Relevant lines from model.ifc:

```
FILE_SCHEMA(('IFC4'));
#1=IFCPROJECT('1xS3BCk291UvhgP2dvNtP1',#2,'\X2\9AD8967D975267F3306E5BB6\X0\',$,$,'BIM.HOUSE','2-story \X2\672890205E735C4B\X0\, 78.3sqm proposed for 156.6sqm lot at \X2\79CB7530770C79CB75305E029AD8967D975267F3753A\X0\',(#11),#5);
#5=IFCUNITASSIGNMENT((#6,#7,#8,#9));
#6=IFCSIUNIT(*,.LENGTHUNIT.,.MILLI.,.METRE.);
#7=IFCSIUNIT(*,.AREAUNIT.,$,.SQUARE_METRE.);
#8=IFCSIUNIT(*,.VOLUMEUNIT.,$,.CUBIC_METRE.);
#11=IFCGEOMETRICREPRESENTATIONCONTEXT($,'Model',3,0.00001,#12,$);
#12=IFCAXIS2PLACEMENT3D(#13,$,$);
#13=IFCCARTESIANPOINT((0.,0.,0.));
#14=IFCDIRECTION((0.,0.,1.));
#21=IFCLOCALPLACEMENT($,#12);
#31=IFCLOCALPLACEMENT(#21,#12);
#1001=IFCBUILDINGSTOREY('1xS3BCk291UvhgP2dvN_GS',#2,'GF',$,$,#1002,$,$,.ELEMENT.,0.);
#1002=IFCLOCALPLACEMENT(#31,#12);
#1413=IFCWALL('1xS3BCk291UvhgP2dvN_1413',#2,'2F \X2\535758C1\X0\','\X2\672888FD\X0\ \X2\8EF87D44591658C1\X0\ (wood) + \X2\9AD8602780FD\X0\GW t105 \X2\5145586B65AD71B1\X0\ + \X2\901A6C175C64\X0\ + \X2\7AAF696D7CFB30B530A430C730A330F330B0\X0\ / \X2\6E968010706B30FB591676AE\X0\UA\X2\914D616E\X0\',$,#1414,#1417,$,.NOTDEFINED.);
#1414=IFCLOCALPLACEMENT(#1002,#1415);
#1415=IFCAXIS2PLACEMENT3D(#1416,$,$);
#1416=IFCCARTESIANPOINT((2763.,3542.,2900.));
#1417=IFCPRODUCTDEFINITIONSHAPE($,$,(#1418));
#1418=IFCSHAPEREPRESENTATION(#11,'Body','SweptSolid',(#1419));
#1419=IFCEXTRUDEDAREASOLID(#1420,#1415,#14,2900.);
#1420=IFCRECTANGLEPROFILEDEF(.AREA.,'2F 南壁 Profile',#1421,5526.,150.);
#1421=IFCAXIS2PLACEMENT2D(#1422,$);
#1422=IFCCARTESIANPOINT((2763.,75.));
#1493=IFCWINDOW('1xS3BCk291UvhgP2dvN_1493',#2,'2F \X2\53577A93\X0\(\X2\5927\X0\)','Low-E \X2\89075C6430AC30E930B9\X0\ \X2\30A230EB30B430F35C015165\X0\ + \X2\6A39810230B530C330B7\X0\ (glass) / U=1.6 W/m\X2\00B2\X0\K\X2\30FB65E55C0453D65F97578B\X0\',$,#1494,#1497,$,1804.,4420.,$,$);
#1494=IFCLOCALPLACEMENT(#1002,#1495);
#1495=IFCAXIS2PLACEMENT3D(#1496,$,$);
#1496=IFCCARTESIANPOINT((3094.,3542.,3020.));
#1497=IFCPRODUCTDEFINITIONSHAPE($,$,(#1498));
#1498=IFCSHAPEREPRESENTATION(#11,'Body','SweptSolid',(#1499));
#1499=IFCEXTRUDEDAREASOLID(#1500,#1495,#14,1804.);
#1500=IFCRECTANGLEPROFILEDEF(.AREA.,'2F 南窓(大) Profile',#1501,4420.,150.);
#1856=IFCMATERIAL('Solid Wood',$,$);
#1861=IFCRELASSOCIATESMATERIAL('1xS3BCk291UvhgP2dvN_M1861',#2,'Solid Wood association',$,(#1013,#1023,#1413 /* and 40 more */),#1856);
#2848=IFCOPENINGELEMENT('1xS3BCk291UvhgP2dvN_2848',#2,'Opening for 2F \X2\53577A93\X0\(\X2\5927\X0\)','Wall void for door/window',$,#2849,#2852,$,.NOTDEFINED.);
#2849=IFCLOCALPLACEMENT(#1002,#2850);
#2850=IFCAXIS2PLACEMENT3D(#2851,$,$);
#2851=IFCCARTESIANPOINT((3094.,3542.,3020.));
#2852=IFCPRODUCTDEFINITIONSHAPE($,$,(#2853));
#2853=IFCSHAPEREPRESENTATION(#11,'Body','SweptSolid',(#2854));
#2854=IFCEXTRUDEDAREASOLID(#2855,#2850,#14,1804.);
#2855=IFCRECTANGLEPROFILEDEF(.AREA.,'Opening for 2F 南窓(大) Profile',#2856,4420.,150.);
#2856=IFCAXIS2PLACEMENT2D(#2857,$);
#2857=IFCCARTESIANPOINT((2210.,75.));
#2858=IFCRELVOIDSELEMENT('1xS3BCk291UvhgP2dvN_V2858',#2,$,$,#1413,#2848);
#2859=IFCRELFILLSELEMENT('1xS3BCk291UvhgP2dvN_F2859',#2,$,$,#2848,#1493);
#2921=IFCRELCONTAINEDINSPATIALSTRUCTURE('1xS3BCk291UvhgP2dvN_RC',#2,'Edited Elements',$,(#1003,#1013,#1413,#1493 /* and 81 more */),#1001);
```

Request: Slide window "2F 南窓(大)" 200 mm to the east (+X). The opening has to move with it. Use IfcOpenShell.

```python
import ifcopenshell
import ifcopenshell.api.geometry
import ifcopenshell.util.placement
import ifcopenshell.util.unit

model = ifcopenshell.open("model.ifc")
unit_scale = ifcopenshell.util.unit.calculate_unit_scale(model)

window = model.by_id(1493)
opening = window.FillsVoids[0].RelatingOpeningElement
wall = opening.VoidsElements[0].RelatingBuildingElement

wall_matrix = ifcopenshell.util.placement.get_local_placement(wall.ObjectPlacement)
shift = wall_matrix[:3, 0] * 0.2 / unit_scale
before = ifcopenshell.util.placement.get_local_placement(window.ObjectPlacement)[:3, 3].copy()

# The window is not placed relative to its opening, so move both.
for product in (opening, window):
    matrix = ifcopenshell.util.placement.get_local_placement(product.ObjectPlacement)
    matrix[:3, 3] += shift
    ifcopenshell.api.geometry.edit_object_placement(model, product=product, matrix=matrix, is_si=False)

after = ifcopenshell.util.placement.get_local_placement(window.ObjectPlacement)[:3, 3]
print("window moved by", (after - before).round(3) + 0.0)

model.write("model-out.ifc")
```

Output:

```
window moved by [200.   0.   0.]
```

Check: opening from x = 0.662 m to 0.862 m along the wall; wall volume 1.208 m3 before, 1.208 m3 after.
